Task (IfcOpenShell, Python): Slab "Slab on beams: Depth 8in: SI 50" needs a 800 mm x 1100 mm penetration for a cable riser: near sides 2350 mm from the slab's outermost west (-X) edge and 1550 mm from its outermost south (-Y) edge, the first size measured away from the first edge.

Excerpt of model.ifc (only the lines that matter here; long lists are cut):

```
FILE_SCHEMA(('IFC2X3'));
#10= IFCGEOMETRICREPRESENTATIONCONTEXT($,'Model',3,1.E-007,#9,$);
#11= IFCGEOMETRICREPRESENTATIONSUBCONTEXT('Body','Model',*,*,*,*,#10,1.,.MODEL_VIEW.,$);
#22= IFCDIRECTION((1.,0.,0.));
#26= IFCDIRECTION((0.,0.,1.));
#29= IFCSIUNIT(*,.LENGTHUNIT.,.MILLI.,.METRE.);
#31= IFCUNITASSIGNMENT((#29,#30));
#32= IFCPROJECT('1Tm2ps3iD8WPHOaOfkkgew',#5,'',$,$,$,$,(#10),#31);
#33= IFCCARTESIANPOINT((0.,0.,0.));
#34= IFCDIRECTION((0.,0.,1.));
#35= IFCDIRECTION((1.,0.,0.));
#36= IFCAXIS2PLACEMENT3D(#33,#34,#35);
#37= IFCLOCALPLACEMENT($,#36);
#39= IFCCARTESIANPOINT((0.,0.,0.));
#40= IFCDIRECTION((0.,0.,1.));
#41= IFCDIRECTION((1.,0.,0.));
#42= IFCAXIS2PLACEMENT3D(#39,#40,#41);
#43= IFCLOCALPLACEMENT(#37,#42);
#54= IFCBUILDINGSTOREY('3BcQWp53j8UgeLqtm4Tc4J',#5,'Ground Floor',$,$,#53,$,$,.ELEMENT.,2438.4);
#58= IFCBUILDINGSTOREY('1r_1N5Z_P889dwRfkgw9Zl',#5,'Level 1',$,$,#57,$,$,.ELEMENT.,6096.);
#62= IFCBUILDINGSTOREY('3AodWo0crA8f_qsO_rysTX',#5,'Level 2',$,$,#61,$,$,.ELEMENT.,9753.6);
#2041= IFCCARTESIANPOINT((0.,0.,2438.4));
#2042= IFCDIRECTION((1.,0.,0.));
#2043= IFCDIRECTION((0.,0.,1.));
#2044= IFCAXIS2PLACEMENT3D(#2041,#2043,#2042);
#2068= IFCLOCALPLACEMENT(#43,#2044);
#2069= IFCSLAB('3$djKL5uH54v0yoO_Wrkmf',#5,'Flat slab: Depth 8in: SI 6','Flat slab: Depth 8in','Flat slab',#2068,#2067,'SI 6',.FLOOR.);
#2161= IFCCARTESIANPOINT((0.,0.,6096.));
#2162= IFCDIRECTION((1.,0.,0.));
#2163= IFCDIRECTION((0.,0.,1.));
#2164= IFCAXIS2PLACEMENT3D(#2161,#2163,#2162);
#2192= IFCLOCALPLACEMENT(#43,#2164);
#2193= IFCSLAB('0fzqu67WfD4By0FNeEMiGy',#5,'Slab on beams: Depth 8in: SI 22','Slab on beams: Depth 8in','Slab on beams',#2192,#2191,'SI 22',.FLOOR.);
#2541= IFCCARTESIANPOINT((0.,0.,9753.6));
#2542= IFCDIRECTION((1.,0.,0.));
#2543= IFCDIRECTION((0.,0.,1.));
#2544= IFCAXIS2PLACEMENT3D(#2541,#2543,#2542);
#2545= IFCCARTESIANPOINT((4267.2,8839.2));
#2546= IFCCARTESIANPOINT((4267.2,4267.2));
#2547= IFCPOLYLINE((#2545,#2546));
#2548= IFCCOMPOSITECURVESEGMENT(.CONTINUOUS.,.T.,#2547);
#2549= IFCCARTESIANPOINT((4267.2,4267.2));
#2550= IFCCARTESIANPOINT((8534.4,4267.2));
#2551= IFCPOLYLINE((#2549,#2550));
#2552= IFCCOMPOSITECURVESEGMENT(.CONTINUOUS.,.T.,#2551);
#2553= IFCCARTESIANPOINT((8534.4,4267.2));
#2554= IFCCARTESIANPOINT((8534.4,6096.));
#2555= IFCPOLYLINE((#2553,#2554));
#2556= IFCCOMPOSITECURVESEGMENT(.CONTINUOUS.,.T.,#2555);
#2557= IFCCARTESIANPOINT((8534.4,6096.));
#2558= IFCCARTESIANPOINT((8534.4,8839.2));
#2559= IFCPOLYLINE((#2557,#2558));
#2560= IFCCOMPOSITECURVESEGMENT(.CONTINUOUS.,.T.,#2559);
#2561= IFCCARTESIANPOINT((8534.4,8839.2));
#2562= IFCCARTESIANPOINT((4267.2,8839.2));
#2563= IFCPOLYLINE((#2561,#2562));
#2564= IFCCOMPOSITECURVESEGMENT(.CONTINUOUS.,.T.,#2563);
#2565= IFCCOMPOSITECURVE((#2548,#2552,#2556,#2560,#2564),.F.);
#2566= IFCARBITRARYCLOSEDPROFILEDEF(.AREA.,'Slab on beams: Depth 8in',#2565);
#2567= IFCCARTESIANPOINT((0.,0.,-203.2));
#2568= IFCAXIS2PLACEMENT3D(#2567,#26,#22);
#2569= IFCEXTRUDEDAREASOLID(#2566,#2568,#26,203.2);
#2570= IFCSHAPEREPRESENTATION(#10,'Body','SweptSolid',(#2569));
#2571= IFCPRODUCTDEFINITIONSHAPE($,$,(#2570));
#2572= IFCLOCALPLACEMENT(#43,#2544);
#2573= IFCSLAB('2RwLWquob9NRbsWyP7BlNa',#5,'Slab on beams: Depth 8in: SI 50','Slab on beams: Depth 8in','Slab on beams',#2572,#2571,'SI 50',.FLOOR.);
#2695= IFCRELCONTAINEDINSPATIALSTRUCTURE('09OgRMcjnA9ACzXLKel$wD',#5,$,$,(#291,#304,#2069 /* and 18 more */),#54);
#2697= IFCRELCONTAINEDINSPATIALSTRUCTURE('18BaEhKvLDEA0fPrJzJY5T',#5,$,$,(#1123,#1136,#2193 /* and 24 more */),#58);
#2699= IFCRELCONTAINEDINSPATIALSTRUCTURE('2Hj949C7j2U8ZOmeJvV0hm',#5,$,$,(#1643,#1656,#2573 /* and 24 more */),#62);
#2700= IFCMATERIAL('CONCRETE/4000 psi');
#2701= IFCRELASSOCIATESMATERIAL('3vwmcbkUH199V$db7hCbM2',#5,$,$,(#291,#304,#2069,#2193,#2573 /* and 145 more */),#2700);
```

```python
import numpy as np
import ifcopenshell
import ifcopenshell.api.feature
import ifcopenshell.api.geometry
import ifcopenshell.api.root
import ifcopenshell.geom
import ifcopenshell.util.placement
import ifcopenshell.util.representation
import ifcopenshell.util.shape
import ifcopenshell.util.unit

model = ifcopenshell.open("model.ifc")
unit_scale = ifcopenshell.util.unit.calculate_unit_scale(model)
settings = ifcopenshell.geom.settings()


def volume(element):
    """Net volume in cubic metres, openings subtracted."""
    shape = ifcopenshell.geom.create_shape(settings, element)
    return ifcopenshell.util.shape.get_volume(shape.geometry)


slab = model.by_id(2573)
before = volume(slab)

# Extent in the slab's own axes, in metres. The edges named are its -X and -Y sides.
slab_shape = ifcopenshell.geom.create_shape(settings, slab)
vertices = ifcopenshell.util.shape.get_vertices(slab_shape.geometry)
x_min, y_min, bottom = vertices.min(axis=0)
top = vertices[:, 2].max()

opening = ifcopenshell.api.root.create_entity(model, ifc_class="IfcOpeningElement", name="Cable riser opening")
context = ifcopenshell.util.representation.get_context(model, "Model", "Body", "MODEL_VIEW")
width, depth = 0.8, 1.1
outline = [(0.0, 0.0), (width, 0.0), (width, depth), (0.0, depth), (0.0, 0.0)]
# Overshoot both faces by 50 mm so the cut is clean.
shape = ifcopenshell.api.geometry.add_slab_representation(
    model, context=context, depth=top - bottom + 0.1, polyline=outline
)
ifcopenshell.api.geometry.assign_representation(model, product=opening, representation=shape)

matrix = ifcopenshell.util.placement.get_local_placement(slab.ObjectPlacement)
matrix[:, 3] = matrix @ np.append(np.array([x_min + 2.35, y_min + 1.55, bottom - 0.05]) / unit_scale, 1.0)
ifcopenshell.api.geometry.edit_object_placement(model, product=opening, matrix=matrix, is_si=False)
ifcopenshell.api.feature.add_feature(model, feature=opening, element=slab)

after = volume(slab)

print(f"slab volume {before:.3f} -> {after:.3f} m3")

model.write("model_edited.ifc")
```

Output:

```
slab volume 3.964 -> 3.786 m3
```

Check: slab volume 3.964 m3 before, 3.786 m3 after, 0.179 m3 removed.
